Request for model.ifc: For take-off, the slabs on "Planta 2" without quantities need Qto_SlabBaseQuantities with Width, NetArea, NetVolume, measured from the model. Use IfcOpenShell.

First a look at what the model holds.

```python
import ifcopenshell
import ifcopenshell.util.element
import ifcopenshell.util.unit

model = ifcopenshell.open("model.ifc")
print(model.schema)
for unit_type in ("LENGTHUNIT", "AREAUNIT", "VOLUMEUNIT"):
    print(unit_type, ifcopenshell.util.unit.calculate_unit_scale(model, unit_type))
storey = next(s for s in model.by_type("IfcBuildingStorey") if s.Name == "Planta 2")
slabs = [e for e in ifcopenshell.util.element.get_decomposition(storey) if e.is_a("IfcSlab")]
for e in sorted(slabs, key=lambda e: e.id()):
    print(e.id(), e.is_a(), e.Name, list(ifcopenshell.util.element.get_psets(e, qtos_only=True)), sep=" | ")
```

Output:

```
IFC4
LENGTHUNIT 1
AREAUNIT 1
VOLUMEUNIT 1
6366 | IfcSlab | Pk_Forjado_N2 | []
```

```python
import ifcopenshell
import ifcopenshell.api.pset
import ifcopenshell.geom
import ifcopenshell.util.element
import ifcopenshell.util.shape
import ifcopenshell.util.unit

model = ifcopenshell.open("model.ifc")
unit_scale = ifcopenshell.util.unit.calculate_unit_scale(model)
area_scale = ifcopenshell.util.unit.calculate_unit_scale(model, "AREAUNIT")
volume_scale = ifcopenshell.util.unit.calculate_unit_scale(model, "VOLUMEUNIT")
settings = ifcopenshell.geom.settings()

storey = next(s for s in model.by_type("IfcBuildingStorey") if s.Name == "Planta 2")
slabs = [e for e in ifcopenshell.util.element.get_decomposition(storey) if e.is_a("IfcSlab")]

for e in sorted(slabs, key=lambda e: e.id()):
    if ifcopenshell.util.element.get_psets(e, qtos_only=True, should_inherit=False):
        continue
    # Geometry comes back in metres, in the element's own axes.
    shape = ifcopenshell.geom.create_shape(settings, e)
    values = {
        "Width": ifcopenshell.util.shape.get_z(shape.geometry) / unit_scale,
        "NetArea": ifcopenshell.util.shape.get_footprint_area(shape.geometry) / area_scale,
        "NetVolume": ifcopenshell.util.shape.get_volume(shape.geometry) / volume_scale,
    }
    qto = ifcopenshell.api.pset.add_qto(model, product=e, name="Qto_SlabBaseQuantities")
    ifcopenshell.api.pset.edit_qto(model, qto=qto, properties=values)
    print(e.id(), {k: round(v, 3) for k, v in values.items()})

model.write("model_v2.ifc")
```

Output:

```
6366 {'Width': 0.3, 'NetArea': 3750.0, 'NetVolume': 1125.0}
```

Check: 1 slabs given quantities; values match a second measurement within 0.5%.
